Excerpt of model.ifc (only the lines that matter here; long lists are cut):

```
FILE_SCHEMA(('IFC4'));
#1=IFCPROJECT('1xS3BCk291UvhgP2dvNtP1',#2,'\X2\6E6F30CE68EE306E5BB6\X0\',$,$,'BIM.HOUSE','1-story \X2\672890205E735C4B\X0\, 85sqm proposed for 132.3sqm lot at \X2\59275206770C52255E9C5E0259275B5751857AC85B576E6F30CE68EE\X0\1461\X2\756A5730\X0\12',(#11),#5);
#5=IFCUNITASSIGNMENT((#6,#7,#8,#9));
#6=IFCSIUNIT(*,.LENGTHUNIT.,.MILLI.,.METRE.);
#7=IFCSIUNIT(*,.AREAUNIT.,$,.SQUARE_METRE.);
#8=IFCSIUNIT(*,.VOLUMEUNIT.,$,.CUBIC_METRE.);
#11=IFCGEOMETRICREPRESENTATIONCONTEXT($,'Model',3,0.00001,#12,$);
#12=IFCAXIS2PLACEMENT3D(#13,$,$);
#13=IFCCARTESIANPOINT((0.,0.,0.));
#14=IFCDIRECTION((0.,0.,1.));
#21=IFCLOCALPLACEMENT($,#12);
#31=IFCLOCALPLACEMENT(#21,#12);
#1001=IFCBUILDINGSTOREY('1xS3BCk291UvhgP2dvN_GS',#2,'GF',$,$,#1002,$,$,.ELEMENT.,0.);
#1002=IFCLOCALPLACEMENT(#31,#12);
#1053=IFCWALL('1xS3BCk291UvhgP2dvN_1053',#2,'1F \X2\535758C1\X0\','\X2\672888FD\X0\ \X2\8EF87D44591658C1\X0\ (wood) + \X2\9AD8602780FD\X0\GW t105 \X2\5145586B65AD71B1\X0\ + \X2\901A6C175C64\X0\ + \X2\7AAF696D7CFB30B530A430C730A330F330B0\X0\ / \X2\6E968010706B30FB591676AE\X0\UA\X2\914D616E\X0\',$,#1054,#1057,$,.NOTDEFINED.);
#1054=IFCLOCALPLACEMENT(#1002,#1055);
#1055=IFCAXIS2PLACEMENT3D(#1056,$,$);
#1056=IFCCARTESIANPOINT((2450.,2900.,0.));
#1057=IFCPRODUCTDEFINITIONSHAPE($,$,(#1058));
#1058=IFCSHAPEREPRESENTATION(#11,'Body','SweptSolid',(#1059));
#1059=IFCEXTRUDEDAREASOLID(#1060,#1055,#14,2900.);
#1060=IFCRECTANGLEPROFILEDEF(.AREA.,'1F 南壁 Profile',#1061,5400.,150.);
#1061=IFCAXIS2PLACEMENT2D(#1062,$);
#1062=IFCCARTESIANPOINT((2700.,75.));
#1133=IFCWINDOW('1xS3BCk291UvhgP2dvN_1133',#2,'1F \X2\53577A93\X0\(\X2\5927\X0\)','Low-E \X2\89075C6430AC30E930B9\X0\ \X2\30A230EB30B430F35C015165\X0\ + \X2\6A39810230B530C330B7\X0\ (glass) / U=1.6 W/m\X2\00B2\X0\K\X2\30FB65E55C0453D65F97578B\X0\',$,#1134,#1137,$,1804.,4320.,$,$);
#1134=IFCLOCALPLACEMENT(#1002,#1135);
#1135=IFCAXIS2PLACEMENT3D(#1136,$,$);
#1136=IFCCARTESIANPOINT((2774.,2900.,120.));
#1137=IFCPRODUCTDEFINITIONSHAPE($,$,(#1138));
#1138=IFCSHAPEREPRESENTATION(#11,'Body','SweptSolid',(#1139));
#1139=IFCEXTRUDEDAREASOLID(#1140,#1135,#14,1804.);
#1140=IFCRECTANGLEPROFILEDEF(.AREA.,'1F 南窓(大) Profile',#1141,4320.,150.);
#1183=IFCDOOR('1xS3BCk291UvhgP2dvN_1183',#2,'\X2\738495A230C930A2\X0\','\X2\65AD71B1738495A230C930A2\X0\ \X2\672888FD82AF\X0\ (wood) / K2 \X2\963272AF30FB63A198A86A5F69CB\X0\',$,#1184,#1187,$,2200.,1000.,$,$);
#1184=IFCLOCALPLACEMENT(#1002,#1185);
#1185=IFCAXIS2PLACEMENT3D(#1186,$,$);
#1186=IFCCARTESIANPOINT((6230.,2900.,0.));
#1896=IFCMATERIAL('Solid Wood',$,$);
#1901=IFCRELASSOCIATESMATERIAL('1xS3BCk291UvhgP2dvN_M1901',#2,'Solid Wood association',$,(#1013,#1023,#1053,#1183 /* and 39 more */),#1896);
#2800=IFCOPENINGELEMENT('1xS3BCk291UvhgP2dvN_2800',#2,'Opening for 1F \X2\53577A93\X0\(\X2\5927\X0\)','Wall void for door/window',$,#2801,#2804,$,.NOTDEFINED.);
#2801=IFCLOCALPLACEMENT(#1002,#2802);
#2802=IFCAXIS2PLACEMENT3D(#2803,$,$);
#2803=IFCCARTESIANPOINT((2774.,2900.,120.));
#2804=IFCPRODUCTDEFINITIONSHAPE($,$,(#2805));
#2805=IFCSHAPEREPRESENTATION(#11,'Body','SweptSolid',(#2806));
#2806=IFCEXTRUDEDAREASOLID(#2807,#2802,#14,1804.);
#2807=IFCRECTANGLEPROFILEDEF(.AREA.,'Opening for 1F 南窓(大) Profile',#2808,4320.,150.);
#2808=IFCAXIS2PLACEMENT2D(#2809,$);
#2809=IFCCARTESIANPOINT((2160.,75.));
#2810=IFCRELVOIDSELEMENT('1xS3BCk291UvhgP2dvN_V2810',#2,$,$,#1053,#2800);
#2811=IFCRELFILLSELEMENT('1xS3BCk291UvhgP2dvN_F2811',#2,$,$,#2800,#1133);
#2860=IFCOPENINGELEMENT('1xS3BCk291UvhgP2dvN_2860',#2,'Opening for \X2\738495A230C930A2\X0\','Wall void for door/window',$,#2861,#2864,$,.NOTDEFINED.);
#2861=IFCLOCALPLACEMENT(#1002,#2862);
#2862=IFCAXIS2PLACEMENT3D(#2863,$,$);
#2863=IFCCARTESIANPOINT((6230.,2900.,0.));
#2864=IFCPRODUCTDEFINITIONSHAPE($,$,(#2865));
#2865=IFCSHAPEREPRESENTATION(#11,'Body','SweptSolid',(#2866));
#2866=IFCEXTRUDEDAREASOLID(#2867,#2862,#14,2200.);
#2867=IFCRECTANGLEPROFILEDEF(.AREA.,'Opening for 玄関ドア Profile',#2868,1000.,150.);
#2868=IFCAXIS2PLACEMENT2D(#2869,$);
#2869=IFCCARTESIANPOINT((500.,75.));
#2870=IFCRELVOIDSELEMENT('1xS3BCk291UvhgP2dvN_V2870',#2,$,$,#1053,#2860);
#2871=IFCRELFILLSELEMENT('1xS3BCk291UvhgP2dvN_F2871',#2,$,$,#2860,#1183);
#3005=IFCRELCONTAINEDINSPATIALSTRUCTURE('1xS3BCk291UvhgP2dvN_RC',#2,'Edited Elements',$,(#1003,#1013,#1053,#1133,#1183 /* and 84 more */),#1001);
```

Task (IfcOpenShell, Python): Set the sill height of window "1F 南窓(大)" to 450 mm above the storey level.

```python
import numpy as np
import ifcopenshell
import ifcopenshell.api.geometry
import ifcopenshell.geom
import ifcopenshell.util.element
import ifcopenshell.util.placement
import ifcopenshell.util.shape
import ifcopenshell.util.unit

model = ifcopenshell.open("model.ifc")
unit_scale = ifcopenshell.util.unit.calculate_unit_scale(model)

window = model.by_guid("1xS3BCk291UvhgP2dvN_1133")
opening = window.FillsVoids[0].RelatingOpeningElement
storey = ifcopenshell.util.element.get_container(window, ifc_class="IfcBuildingStorey")
level = ifcopenshell.util.placement.get_local_placement(storey.ObjectPlacement)[2, 3]

# The opening's origin need not be at the sill, so measure its lowest point.
shape = ifcopenshell.geom.create_shape(ifcopenshell.geom.settings(), opening)
bottom = ifcopenshell.util.shape.get_shape_bottom_elevation(shape, shape.geometry) / unit_scale
dz = level + 450.0 - bottom

shift = np.array([0.0, 0.0, dz])
# The window is not placed relative to its opening, so move both.
for product in (opening, window):
    matrix = ifcopenshell.util.placement.get_local_placement(product.ObjectPlacement)
    matrix[:3, 3] += shift
    ifcopenshell.api.geometry.edit_object_placement(model, product=product, matrix=matrix, is_si=False)

print(f"moved by {dz * unit_scale:+.3f} m")

model.write("model-out.ifc")
```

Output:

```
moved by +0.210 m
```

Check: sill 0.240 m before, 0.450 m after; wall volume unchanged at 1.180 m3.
